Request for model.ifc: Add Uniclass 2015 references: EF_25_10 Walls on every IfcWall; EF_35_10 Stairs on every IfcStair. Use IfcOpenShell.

First a look at what the model holds.

```python
import ifcopenshell

model = ifcopenshell.open("model.ifc")
print(model.schema)
print("classifications:", [c.Name for c in model.by_type("IfcClassification")])
for ifc_class in ("IfcDoor", "IfcRoof", "IfcStair", "IfcWall", "IfcWindow"):
    print(ifc_class, len(model.by_type(ifc_class)))
```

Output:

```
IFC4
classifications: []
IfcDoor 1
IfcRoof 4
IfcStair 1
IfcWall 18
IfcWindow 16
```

```python
import ifcopenshell
import ifcopenshell.api.classification

model = ifcopenshell.open("model.ifc")

system = ifcopenshell.api.classification.add_classification(model, classification="Uniclass 2015")

codes = {
    "IfcWall": ("EF_25_10", "Walls"),
    "IfcStair": ("EF_35_10", "Stairs"),
}
for ifc_class, (code, name) in codes.items():
    products = model.by_type(ifc_class)
    ifcopenshell.api.classification.add_reference(
        model, products=products, classification=system, identification=code, name=name
    )
    print(code, len(products))

model.write("model_rev.ifc")
```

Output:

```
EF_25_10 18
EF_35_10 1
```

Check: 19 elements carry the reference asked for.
